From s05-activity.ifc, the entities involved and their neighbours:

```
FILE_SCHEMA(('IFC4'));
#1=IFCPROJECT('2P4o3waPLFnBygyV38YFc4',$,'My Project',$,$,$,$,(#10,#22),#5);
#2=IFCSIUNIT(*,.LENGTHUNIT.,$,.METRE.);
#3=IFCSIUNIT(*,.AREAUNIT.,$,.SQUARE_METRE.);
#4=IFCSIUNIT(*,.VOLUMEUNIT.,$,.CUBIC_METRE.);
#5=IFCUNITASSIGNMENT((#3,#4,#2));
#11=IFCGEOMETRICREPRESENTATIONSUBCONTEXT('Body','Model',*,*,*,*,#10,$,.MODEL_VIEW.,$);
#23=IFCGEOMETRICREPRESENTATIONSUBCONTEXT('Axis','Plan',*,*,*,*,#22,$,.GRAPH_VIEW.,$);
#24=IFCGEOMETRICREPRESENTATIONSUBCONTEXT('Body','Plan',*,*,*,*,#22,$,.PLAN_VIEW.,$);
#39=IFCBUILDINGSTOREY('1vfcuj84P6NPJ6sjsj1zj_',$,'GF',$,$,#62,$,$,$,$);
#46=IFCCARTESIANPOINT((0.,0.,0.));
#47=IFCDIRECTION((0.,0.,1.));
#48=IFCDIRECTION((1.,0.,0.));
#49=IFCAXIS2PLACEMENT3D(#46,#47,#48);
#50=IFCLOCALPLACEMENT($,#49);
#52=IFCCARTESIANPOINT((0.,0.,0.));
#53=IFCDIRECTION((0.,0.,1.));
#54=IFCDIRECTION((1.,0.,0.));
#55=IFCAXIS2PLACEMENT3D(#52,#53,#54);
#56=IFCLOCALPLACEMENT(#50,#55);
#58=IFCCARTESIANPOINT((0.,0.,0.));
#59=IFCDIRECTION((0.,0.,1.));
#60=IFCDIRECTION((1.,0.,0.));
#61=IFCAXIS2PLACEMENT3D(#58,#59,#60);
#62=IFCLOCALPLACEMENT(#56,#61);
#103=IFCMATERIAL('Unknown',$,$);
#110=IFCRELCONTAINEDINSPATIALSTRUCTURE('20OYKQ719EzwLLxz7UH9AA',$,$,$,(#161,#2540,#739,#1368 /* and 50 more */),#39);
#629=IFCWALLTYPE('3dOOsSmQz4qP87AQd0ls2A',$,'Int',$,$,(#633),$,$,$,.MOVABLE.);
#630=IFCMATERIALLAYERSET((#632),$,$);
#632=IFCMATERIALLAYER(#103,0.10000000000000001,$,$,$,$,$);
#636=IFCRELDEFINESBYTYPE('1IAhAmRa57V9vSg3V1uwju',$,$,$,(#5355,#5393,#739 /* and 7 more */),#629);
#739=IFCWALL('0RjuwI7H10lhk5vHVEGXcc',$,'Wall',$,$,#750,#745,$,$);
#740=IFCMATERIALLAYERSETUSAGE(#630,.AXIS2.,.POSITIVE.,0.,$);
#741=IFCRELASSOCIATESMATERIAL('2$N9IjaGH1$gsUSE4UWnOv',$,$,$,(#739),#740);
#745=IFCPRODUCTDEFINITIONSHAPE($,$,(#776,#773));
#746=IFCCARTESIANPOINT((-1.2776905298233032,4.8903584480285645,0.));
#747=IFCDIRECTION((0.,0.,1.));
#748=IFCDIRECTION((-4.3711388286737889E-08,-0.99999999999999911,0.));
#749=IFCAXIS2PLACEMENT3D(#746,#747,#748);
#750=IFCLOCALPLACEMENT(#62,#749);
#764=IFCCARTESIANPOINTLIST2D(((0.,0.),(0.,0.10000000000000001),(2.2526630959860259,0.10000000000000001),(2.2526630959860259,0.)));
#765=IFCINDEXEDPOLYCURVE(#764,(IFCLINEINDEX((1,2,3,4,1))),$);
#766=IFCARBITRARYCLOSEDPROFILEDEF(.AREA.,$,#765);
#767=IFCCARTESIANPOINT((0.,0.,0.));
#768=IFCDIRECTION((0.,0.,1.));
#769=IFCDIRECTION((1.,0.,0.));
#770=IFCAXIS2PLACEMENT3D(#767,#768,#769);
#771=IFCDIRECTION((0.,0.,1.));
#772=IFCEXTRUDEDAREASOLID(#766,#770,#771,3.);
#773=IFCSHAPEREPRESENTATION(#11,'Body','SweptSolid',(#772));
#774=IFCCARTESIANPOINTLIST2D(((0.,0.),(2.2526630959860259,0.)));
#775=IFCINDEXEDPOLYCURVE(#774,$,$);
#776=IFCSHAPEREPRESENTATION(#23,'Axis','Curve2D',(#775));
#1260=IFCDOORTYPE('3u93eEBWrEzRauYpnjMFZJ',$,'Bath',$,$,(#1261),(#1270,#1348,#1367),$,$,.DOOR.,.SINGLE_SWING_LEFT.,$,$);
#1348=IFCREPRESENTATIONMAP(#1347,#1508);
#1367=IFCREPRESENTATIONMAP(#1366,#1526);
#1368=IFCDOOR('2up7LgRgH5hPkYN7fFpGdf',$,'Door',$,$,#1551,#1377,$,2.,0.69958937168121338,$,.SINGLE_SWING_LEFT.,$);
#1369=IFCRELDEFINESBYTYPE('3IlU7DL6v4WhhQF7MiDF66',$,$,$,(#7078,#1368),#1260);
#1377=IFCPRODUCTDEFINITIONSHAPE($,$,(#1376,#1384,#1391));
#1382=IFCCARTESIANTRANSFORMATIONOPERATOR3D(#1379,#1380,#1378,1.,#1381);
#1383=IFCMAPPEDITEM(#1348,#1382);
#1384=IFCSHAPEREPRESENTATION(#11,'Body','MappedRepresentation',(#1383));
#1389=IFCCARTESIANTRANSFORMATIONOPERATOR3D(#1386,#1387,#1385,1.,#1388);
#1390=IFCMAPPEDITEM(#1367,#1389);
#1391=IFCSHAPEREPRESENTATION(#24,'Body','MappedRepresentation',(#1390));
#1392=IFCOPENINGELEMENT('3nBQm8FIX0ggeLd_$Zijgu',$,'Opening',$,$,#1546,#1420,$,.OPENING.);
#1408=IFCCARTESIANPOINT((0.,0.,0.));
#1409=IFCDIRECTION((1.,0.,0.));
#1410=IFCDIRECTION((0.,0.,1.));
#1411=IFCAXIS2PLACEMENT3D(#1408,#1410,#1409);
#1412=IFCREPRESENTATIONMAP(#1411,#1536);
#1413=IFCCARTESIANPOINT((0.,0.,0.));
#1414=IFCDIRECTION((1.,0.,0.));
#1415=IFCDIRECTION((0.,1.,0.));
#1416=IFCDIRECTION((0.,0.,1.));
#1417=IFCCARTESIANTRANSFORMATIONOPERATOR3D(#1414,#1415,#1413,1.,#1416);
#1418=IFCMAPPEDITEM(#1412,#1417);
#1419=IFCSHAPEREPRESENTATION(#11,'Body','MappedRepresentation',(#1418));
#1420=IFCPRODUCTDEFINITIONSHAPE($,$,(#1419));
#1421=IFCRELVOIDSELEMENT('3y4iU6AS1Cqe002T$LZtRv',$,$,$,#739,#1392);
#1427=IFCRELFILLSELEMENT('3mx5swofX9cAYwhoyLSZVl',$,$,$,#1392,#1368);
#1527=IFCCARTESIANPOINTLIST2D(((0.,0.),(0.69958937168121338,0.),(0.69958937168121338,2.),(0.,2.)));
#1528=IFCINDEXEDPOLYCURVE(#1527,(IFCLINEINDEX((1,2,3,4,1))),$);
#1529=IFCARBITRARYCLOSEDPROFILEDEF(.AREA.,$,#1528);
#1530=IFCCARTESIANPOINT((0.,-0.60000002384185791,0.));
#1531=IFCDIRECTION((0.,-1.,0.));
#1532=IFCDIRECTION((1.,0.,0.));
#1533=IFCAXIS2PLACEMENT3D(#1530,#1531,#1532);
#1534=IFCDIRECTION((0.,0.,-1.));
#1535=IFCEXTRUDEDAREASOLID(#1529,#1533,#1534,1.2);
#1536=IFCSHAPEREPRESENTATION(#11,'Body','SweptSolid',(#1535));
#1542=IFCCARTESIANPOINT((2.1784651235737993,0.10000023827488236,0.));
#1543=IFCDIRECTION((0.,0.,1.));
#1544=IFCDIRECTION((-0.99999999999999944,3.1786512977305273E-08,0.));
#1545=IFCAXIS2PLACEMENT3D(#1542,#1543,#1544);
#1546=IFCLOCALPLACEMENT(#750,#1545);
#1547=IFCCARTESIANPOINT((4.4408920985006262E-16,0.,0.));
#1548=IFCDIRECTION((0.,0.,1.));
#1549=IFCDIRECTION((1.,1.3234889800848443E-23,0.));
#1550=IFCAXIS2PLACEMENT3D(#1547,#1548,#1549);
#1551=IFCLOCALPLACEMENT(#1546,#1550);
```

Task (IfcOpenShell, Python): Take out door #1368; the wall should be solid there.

```python
import ifcopenshell
import ifcopenshell.api.feature
import ifcopenshell.api.root
import ifcopenshell.geom
import ifcopenshell.util.shape

model = ifcopenshell.open("s05-activity.ifc")
settings = ifcopenshell.geom.settings()


def volume(element):
    """Net volume in cubic metres, openings subtracted."""
    shape = ifcopenshell.geom.create_shape(settings, element)
    return ifcopenshell.util.shape.get_volume(shape.geometry)


door = model.by_guid("2up7LgRgH5hPkYN7fFpGdf")
opening = door.FillsVoids[0].RelatingOpeningElement
wall = opening.VoidsElements[0].RelatingBuildingElement
before = volume(wall)

ifcopenshell.api.root.remove_product(model, product=door)
ifcopenshell.api.feature.remove_feature(model, feature=opening)

after = volume(wall)

print(f"wall volume {before:.3f} -> {after:.3f} m3")

model.write("s05-activity_edited.ifc")
```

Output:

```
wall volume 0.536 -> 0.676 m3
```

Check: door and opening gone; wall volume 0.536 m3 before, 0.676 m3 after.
